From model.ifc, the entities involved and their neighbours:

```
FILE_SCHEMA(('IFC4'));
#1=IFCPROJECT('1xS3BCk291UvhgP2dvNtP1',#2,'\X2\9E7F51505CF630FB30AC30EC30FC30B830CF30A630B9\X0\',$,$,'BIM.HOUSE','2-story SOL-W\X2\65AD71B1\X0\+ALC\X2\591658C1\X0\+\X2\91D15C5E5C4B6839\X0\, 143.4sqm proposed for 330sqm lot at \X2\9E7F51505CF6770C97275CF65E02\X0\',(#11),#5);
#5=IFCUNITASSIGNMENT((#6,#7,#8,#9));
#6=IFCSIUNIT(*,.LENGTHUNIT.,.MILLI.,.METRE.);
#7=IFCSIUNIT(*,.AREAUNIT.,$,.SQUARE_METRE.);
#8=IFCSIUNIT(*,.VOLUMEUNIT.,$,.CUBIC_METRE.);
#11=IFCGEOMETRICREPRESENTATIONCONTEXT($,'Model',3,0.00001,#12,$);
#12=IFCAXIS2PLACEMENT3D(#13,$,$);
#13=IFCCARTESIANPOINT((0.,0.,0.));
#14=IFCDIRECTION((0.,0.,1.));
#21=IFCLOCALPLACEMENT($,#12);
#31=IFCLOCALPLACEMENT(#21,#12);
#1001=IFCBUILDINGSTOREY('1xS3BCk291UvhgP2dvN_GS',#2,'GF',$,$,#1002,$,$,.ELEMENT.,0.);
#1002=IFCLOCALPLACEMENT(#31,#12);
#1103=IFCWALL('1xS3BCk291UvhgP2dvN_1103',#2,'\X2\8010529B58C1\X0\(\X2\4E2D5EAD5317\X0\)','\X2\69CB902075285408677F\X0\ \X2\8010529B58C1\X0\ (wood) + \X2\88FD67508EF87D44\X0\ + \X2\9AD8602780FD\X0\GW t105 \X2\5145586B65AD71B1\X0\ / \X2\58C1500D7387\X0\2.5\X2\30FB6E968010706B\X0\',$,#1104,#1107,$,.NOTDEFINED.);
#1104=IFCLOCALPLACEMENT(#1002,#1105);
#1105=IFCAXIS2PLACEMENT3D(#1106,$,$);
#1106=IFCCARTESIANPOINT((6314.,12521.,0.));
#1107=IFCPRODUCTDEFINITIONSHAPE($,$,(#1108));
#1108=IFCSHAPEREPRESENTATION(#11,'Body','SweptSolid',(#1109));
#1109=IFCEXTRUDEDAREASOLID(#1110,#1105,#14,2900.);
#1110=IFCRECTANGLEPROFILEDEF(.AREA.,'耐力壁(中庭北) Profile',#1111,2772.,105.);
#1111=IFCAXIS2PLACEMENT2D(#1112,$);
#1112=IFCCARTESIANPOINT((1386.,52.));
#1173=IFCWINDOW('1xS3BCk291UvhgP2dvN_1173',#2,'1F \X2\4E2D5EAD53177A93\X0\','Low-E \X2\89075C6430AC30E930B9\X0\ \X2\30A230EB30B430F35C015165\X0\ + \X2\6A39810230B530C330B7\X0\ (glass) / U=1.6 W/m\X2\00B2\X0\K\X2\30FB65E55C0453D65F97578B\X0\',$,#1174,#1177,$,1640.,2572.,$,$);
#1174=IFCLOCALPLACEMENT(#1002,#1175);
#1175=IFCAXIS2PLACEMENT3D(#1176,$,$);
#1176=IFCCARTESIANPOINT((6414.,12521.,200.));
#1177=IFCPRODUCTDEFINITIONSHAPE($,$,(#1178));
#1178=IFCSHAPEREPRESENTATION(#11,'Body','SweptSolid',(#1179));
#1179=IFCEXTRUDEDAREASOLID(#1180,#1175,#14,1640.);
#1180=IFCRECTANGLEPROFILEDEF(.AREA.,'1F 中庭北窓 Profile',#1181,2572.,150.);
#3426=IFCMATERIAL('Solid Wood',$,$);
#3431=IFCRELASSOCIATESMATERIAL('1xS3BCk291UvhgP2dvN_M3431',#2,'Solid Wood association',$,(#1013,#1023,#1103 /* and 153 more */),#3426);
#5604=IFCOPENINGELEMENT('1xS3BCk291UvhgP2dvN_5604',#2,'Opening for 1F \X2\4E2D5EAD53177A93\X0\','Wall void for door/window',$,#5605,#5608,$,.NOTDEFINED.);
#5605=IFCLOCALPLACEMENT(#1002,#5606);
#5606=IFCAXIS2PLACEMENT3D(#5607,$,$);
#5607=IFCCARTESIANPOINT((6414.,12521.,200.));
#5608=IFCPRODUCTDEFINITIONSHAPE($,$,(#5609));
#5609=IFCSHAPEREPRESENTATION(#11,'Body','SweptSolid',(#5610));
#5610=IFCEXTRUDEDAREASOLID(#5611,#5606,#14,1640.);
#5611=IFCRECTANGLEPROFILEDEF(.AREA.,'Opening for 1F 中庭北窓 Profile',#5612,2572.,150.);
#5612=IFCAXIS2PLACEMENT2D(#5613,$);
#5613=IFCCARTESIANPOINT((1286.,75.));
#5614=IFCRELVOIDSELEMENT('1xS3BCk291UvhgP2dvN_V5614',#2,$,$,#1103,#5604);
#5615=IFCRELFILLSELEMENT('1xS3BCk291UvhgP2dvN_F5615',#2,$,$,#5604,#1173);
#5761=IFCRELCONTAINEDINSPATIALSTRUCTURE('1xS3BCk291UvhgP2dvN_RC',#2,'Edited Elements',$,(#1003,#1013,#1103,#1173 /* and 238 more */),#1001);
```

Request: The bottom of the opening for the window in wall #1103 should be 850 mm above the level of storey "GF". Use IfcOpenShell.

```python
import numpy as np
import ifcopenshell
import ifcopenshell.api.geometry
import ifcopenshell.geom
import ifcopenshell.util.element
import ifcopenshell.util.placement
import ifcopenshell.util.shape
import ifcopenshell.util.unit

model = ifcopenshell.open("model.ifc")
unit_scale = ifcopenshell.util.unit.calculate_unit_scale(model)

window = model.by_guid("1xS3BCk291UvhgP2dvN_1173")
opening = window.FillsVoids[0].RelatingOpeningElement
storey = ifcopenshell.util.element.get_container(window, ifc_class="IfcBuildingStorey")
level = ifcopenshell.util.placement.get_local_placement(storey.ObjectPlacement)[2, 3]

# The opening's origin need not be at the sill, so measure its lowest point.
shape = ifcopenshell.geom.create_shape(ifcopenshell.geom.settings(), opening)
bottom = ifcopenshell.util.shape.get_shape_bottom_elevation(shape, shape.geometry) / unit_scale
dz = level + 0.85 / unit_scale - bottom

shift = np.array([0.0, 0.0, dz])
# The window is not placed relative to its opening, so move both.
for product in (opening, window):
    matrix = ifcopenshell.util.placement.get_local_placement(product.ObjectPlacement)
    matrix[:3, 3] += shift
    ifcopenshell.api.geometry.edit_object_placement(model, product=product, matrix=matrix, is_si=False)

print(f"moved by {dz * unit_scale:+.3f} m")

model.write("model_updated.ifc")
```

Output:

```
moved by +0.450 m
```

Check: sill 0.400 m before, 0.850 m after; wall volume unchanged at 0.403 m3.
